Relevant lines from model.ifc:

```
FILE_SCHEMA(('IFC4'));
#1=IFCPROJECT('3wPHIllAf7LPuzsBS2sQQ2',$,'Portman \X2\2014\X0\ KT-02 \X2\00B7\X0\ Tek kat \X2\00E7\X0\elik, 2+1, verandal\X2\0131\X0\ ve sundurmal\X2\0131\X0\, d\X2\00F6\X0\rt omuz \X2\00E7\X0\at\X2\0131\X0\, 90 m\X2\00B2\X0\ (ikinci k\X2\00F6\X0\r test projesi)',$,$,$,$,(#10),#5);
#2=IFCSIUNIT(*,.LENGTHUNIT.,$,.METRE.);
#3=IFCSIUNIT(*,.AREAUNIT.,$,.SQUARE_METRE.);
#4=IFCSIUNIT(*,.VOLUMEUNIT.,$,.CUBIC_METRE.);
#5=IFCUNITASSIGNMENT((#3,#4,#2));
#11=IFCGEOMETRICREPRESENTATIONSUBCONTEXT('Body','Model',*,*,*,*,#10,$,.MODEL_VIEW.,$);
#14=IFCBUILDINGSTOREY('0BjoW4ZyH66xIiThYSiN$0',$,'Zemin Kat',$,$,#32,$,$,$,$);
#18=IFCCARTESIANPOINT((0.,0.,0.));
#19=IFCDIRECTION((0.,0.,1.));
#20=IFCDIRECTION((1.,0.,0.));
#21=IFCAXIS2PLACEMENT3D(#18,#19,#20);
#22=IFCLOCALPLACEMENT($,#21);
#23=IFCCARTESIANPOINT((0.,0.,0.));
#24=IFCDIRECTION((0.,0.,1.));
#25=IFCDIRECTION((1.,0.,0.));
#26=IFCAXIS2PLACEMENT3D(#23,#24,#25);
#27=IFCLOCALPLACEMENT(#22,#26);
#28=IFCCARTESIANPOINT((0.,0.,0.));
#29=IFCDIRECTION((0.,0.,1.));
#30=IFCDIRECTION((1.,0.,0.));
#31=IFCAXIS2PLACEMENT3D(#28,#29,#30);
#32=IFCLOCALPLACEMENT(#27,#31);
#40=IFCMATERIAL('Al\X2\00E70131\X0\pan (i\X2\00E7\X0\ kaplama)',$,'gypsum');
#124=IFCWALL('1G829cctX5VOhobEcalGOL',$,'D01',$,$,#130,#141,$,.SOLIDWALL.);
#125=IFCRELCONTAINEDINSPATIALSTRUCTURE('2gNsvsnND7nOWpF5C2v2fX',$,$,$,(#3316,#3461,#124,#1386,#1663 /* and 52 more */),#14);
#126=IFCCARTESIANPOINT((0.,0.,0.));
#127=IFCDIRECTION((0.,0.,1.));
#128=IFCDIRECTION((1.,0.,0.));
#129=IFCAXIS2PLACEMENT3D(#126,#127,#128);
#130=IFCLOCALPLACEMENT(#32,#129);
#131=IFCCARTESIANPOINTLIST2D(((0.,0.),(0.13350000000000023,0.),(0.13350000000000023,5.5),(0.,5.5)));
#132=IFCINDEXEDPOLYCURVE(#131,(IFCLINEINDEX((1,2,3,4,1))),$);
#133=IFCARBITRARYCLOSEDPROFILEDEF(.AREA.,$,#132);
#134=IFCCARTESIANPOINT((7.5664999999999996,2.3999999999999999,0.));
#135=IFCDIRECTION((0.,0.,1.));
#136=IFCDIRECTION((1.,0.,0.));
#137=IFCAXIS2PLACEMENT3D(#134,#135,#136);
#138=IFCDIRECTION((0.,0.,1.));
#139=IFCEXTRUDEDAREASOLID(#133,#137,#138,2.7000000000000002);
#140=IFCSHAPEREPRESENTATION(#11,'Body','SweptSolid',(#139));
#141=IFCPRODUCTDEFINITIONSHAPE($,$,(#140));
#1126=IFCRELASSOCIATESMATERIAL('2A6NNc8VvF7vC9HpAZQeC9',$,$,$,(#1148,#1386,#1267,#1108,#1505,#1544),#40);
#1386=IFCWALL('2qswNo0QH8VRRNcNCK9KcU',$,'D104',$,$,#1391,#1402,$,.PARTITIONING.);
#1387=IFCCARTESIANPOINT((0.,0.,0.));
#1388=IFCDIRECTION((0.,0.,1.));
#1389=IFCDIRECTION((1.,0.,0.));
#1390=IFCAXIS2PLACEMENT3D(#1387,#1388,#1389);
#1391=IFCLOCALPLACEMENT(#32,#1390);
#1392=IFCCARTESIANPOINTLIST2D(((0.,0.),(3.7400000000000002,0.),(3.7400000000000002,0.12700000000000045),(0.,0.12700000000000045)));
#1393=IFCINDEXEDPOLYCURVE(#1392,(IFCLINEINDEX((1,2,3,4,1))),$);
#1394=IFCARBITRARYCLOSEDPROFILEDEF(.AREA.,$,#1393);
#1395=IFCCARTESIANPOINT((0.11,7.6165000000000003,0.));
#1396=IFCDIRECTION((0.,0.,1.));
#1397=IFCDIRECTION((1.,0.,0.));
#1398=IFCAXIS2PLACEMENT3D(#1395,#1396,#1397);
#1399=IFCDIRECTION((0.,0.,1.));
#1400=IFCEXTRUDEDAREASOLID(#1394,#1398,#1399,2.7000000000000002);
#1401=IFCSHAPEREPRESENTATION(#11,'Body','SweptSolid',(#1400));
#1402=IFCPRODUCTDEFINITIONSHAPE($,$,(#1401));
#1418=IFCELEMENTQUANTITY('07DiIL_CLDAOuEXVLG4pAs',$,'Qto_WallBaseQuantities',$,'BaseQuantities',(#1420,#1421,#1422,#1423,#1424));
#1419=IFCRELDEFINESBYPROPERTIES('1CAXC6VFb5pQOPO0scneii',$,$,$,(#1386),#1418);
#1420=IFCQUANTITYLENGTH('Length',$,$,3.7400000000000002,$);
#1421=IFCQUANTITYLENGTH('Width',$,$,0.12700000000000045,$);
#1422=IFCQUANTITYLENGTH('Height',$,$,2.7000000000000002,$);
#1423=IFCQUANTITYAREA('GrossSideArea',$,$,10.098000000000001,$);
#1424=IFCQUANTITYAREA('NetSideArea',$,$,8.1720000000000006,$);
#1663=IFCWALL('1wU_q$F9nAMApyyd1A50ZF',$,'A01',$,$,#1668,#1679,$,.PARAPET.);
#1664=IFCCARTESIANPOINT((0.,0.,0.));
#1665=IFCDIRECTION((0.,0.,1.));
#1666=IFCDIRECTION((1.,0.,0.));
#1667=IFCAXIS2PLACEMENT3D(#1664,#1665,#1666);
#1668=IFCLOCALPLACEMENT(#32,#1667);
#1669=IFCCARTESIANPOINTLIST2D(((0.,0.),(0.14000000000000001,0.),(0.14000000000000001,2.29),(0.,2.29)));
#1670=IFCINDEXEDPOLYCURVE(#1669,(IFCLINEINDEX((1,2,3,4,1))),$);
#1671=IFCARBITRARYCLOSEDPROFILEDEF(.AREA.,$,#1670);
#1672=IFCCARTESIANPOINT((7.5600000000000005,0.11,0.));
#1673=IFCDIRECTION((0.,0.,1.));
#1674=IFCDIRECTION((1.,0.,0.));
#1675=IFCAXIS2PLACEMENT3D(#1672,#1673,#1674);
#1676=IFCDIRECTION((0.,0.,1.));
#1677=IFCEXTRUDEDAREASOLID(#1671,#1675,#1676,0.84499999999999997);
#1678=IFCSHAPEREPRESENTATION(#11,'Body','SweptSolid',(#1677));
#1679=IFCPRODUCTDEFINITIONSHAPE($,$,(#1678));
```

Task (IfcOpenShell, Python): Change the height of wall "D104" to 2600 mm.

```python
import ifcopenshell
import ifcopenshell.api.pset
import ifcopenshell.geom
import ifcopenshell.util.element
import ifcopenshell.util.representation
import ifcopenshell.util.shape
import ifcopenshell.util.unit

model = ifcopenshell.open("model.ifc")
unit_scale = ifcopenshell.util.unit.calculate_unit_scale(model)
area_scale = ifcopenshell.util.unit.calculate_unit_scale(model, "AREAUNIT")
settings = ifcopenshell.geom.settings()


def volume(element):
    """Net volume in cubic metres, openings subtracted."""
    shape = ifcopenshell.geom.create_shape(settings, element)
    return ifcopenshell.util.shape.get_volume(shape.geometry)


wall = model.by_guid("2qswNo0QH8VRRNcNCK9KcU")
before = volume(wall)

body = ifcopenshell.util.representation.get_representation(wall, "Model", "Body")
solid = body.Items[0]
old_height = solid.Depth
solid.Depth = 2.6 / unit_scale
after = volume(wall)
thickness = 0.127  # wall thickness in metres

# Update the stored height, areas and volumes.
qto = model.by_id(ifcopenshell.util.element.get_pset(wall, "Qto_WallBaseQuantities", should_inherit=False)["id"])
ifcopenshell.api.pset.edit_qto(model, qto=qto, properties={
    "Height": solid.Depth,
    "GrossSideArea": ifcopenshell.util.element.get_pset(wall, "Qto_WallBaseQuantities", "GrossSideArea") * solid.Depth / old_height,
    "NetSideArea": after / thickness / area_scale,
})

print(f"height {old_height:g} -> {solid.Depth:g}, volume {before:.3f} -> {after:.3f} m3")

model.write("model_rev.ifc")
```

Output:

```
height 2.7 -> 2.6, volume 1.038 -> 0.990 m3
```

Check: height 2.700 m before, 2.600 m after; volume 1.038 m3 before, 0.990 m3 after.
